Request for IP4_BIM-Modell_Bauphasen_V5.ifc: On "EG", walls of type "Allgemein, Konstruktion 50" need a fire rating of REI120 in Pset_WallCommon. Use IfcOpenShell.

First a look at what the model holds.

```python
import ifcopenshell
import ifcopenshell.util.element

model = ifcopenshell.open("IP4_BIM-Modell_Bauphasen_V5.ifc")
print(model.schema)
storey = next(s for s in model.by_type("IfcBuildingStorey") if s.Name == "EG")
walls = [e for e in ifcopenshell.util.element.get_decomposition(storey) if e.is_a("IfcWall")]
seen = {}
for e in walls:
    element_type = ifcopenshell.util.element.get_type(e)
    key = (element_type.Name if element_type != e and element_type else None, ifcopenshell.util.element.get_pset(e, "Pset_WallCommon", "FireRating"))
    seen[key] = seen.get(key, 0) + 1
for (name, value), count in sorted(seen.items(), key=str):
    print(count, "x", name, "|", value)
```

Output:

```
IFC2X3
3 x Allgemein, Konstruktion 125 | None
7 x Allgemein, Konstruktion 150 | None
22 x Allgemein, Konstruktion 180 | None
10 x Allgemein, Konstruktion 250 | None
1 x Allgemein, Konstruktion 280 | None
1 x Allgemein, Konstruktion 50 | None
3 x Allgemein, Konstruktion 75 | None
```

```python
import ifcopenshell
import ifcopenshell.api.pset
import ifcopenshell.util.element

model = ifcopenshell.open("IP4_BIM-Modell_Bauphasen_V5.ifc")

storey = next(s for s in model.by_type("IfcBuildingStorey") if s.Name == "EG")
walls = [e for e in ifcopenshell.util.element.get_decomposition(storey) if e.is_a("IfcWall")]

count = 0
for e in walls:
    element_type = ifcopenshell.util.element.get_type(e)
    if element_type in (None, e) or element_type.Name != "Allgemein, Konstruktion 50":
        continue
    # add_pset returns the element's existing set when there is one.
    pset = ifcopenshell.api.pset.add_pset(model, product=e, name="Pset_WallCommon")
    ifcopenshell.api.pset.edit_pset(model, pset=pset, properties={"FireRating": "REI120"})
    count += 1

print(count, "walls updated")

model.write("IP4_BIM-Modell_Bauphasen_V5_v2.ifc")
```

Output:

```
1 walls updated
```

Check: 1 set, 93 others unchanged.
